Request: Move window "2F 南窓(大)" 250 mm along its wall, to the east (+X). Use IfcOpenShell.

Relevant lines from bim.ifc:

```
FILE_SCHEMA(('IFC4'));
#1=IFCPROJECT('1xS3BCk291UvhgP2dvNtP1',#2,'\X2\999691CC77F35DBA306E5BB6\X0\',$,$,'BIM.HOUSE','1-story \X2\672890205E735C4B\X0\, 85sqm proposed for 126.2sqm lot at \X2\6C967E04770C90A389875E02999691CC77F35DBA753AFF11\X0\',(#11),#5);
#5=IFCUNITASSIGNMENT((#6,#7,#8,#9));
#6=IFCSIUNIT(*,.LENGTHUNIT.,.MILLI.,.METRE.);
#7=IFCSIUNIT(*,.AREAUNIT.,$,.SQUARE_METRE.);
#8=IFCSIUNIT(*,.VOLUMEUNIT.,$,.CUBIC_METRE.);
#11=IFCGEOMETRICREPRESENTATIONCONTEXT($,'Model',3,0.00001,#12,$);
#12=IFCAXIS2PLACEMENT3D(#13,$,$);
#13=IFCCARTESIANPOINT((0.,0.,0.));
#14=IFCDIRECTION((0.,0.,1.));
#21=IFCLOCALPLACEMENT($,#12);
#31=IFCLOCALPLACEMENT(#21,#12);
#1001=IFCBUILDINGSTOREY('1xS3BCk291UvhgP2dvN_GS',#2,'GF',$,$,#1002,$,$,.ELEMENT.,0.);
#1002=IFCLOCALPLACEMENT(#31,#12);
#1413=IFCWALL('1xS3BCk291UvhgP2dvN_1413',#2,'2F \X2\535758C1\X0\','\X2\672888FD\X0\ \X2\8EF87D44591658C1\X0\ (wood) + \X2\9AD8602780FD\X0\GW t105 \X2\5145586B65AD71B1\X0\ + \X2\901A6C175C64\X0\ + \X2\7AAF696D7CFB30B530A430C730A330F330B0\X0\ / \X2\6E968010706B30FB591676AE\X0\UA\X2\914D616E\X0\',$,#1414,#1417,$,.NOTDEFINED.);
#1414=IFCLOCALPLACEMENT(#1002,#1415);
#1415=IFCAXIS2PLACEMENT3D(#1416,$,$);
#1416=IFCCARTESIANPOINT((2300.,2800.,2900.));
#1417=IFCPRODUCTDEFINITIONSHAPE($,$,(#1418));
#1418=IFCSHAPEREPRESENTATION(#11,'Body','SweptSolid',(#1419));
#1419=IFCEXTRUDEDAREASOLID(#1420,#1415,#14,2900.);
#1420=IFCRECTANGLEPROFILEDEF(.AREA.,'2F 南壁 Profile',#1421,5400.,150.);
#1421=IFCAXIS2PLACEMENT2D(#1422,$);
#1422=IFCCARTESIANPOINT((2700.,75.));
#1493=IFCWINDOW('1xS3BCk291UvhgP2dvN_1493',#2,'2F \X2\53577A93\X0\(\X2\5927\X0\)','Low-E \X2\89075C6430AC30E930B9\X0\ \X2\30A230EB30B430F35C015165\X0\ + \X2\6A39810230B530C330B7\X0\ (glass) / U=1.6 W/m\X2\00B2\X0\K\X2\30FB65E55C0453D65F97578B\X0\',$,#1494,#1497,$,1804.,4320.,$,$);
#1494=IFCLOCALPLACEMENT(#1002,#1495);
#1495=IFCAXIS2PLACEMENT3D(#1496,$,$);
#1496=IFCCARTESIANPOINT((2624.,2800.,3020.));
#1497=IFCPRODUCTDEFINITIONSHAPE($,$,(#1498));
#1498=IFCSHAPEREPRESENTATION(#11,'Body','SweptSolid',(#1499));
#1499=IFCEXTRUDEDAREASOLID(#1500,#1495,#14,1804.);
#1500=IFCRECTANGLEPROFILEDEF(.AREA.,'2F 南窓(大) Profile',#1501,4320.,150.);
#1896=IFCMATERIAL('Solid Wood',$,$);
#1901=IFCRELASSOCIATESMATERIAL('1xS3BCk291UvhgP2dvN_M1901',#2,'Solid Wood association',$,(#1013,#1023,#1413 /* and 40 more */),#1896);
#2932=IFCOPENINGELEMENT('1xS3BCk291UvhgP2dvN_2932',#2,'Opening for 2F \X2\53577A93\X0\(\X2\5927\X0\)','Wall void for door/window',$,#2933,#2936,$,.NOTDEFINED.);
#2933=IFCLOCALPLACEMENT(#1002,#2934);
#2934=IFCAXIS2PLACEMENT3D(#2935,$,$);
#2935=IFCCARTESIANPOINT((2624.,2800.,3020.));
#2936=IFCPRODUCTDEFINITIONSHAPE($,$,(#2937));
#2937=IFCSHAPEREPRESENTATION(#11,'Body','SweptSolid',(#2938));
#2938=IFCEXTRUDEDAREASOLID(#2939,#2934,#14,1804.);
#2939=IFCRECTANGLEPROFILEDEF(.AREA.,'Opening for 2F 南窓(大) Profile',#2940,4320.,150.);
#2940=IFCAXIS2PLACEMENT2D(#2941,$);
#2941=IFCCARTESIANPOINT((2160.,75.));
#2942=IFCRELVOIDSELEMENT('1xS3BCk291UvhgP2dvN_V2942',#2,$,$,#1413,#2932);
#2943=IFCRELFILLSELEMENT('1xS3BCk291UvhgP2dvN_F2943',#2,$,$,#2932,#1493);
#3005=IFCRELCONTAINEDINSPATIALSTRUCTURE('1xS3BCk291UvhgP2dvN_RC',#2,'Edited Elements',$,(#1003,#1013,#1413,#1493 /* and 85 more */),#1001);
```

```python
import ifcopenshell
import ifcopenshell.api.geometry
import ifcopenshell.util.placement

model = ifcopenshell.open("bim.ifc")

window = model.by_guid("1xS3BCk291UvhgP2dvN_1493")
opening = window.FillsVoids[0].RelatingOpeningElement
wall = opening.VoidsElements[0].RelatingBuildingElement

wall_matrix = ifcopenshell.util.placement.get_local_placement(wall.ObjectPlacement)
shift = wall_matrix[:3, 0] * 250.0
before = ifcopenshell.util.placement.get_local_placement(window.ObjectPlacement)[:3, 3].copy()

# The window is not placed relative to its opening, so move both.
for product in (opening, window):
    matrix = ifcopenshell.util.placement.get_local_placement(product.ObjectPlacement)
    matrix[:3, 3] += shift
    ifcopenshell.api.geometry.edit_object_placement(model, product=product, matrix=matrix, is_si=False)

after = ifcopenshell.util.placement.get_local_placement(window.ObjectPlacement)[:3, 3]
print("window moved by", (after - before).round(3) + 0.0)

model.write("bim_updated.ifc")
```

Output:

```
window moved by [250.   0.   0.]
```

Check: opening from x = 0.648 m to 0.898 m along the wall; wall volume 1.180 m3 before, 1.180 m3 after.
